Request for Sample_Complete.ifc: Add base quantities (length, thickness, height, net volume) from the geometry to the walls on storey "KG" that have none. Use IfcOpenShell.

First a look at what the model holds.

```python
import ifcopenshell
import ifcopenshell.util.element
import ifcopenshell.util.unit

model = ifcopenshell.open("Sample_Complete.ifc")
print(model.schema)
for unit_type in ("LENGTHUNIT", "AREAUNIT", "VOLUMEUNIT"):
    print(unit_type, ifcopenshell.util.unit.calculate_unit_scale(model, unit_type))
storey = next(s for s in model.by_type("IfcBuildingStorey") if s.Name == "KG")
walls = [e for e in ifcopenshell.util.element.get_decomposition(storey) if e.is_a("IfcWall")]
for e in sorted(walls, key=lambda e: e.id()):
    print(e.id(), e.is_a(), e.Name, list(ifcopenshell.util.element.get_psets(e, qtos_only=True)), sep=" | ")
```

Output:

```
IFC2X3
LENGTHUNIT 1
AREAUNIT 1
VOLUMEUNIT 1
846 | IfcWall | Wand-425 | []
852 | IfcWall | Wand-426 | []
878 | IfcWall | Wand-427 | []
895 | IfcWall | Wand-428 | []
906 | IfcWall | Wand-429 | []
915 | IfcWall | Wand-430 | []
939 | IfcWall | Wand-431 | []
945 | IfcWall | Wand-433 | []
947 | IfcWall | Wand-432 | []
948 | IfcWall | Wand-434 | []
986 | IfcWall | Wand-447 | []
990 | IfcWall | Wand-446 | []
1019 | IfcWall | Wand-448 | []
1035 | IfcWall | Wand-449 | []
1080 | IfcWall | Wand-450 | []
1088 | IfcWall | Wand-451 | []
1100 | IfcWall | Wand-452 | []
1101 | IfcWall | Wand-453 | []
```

```python
import ifcopenshell
import ifcopenshell.api.pset
import ifcopenshell.geom
import ifcopenshell.util.element
import ifcopenshell.util.shape
import ifcopenshell.util.unit

model = ifcopenshell.open("Sample_Complete.ifc")
unit_scale = ifcopenshell.util.unit.calculate_unit_scale(model)
volume_scale = ifcopenshell.util.unit.calculate_unit_scale(model, "VOLUMEUNIT")
settings = ifcopenshell.geom.settings()

storey = next(s for s in model.by_type("IfcBuildingStorey") if s.Name == "KG")
walls = [e for e in ifcopenshell.util.element.get_decomposition(storey) if e.is_a("IfcWall")]

for e in sorted(walls, key=lambda e: e.id()):
    if ifcopenshell.util.element.get_psets(e, qtos_only=True, should_inherit=False):
        continue
    # Geometry comes back in metres, in the element's own axes.
    shape = ifcopenshell.geom.create_shape(settings, e)
    values = {
        "Length": ifcopenshell.util.shape.get_x(shape.geometry) / unit_scale,
        "Width": ifcopenshell.util.shape.get_y(shape.geometry) / unit_scale,
        "Height": ifcopenshell.util.shape.get_z(shape.geometry) / unit_scale,
        "NetVolume": ifcopenshell.util.shape.get_volume(shape.geometry) / volume_scale,
    }
    qto = ifcopenshell.api.pset.add_qto(model, product=e, name="BaseQuantities")
    ifcopenshell.api.pset.edit_qto(model, qto=qto, properties=values)
    print(e.id(), {k: round(v, 3) for k, v in values.items()})

model.write("Sample_Complete_v2.ifc")
```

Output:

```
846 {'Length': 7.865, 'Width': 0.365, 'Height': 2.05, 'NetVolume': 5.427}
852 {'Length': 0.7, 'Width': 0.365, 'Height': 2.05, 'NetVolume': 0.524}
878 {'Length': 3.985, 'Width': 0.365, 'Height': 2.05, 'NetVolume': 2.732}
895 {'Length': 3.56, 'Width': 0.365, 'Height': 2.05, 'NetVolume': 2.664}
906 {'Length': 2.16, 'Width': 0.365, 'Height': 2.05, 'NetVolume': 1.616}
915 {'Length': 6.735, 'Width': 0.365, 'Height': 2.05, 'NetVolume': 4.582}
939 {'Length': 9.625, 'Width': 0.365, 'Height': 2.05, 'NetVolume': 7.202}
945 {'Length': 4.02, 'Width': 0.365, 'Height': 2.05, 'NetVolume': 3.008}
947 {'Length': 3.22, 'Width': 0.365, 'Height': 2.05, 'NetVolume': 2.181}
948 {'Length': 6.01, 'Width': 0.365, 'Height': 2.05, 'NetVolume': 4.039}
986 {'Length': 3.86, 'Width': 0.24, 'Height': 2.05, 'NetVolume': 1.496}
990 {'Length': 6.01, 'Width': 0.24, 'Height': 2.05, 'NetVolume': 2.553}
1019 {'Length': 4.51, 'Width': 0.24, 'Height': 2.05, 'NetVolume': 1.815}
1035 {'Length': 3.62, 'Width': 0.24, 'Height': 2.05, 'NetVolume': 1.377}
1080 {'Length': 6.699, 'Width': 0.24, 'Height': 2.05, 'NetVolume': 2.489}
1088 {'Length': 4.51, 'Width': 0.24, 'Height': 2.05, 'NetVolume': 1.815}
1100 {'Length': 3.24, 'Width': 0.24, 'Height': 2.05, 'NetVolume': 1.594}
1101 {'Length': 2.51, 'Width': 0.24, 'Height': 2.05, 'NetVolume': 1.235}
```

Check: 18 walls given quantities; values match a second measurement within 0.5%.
